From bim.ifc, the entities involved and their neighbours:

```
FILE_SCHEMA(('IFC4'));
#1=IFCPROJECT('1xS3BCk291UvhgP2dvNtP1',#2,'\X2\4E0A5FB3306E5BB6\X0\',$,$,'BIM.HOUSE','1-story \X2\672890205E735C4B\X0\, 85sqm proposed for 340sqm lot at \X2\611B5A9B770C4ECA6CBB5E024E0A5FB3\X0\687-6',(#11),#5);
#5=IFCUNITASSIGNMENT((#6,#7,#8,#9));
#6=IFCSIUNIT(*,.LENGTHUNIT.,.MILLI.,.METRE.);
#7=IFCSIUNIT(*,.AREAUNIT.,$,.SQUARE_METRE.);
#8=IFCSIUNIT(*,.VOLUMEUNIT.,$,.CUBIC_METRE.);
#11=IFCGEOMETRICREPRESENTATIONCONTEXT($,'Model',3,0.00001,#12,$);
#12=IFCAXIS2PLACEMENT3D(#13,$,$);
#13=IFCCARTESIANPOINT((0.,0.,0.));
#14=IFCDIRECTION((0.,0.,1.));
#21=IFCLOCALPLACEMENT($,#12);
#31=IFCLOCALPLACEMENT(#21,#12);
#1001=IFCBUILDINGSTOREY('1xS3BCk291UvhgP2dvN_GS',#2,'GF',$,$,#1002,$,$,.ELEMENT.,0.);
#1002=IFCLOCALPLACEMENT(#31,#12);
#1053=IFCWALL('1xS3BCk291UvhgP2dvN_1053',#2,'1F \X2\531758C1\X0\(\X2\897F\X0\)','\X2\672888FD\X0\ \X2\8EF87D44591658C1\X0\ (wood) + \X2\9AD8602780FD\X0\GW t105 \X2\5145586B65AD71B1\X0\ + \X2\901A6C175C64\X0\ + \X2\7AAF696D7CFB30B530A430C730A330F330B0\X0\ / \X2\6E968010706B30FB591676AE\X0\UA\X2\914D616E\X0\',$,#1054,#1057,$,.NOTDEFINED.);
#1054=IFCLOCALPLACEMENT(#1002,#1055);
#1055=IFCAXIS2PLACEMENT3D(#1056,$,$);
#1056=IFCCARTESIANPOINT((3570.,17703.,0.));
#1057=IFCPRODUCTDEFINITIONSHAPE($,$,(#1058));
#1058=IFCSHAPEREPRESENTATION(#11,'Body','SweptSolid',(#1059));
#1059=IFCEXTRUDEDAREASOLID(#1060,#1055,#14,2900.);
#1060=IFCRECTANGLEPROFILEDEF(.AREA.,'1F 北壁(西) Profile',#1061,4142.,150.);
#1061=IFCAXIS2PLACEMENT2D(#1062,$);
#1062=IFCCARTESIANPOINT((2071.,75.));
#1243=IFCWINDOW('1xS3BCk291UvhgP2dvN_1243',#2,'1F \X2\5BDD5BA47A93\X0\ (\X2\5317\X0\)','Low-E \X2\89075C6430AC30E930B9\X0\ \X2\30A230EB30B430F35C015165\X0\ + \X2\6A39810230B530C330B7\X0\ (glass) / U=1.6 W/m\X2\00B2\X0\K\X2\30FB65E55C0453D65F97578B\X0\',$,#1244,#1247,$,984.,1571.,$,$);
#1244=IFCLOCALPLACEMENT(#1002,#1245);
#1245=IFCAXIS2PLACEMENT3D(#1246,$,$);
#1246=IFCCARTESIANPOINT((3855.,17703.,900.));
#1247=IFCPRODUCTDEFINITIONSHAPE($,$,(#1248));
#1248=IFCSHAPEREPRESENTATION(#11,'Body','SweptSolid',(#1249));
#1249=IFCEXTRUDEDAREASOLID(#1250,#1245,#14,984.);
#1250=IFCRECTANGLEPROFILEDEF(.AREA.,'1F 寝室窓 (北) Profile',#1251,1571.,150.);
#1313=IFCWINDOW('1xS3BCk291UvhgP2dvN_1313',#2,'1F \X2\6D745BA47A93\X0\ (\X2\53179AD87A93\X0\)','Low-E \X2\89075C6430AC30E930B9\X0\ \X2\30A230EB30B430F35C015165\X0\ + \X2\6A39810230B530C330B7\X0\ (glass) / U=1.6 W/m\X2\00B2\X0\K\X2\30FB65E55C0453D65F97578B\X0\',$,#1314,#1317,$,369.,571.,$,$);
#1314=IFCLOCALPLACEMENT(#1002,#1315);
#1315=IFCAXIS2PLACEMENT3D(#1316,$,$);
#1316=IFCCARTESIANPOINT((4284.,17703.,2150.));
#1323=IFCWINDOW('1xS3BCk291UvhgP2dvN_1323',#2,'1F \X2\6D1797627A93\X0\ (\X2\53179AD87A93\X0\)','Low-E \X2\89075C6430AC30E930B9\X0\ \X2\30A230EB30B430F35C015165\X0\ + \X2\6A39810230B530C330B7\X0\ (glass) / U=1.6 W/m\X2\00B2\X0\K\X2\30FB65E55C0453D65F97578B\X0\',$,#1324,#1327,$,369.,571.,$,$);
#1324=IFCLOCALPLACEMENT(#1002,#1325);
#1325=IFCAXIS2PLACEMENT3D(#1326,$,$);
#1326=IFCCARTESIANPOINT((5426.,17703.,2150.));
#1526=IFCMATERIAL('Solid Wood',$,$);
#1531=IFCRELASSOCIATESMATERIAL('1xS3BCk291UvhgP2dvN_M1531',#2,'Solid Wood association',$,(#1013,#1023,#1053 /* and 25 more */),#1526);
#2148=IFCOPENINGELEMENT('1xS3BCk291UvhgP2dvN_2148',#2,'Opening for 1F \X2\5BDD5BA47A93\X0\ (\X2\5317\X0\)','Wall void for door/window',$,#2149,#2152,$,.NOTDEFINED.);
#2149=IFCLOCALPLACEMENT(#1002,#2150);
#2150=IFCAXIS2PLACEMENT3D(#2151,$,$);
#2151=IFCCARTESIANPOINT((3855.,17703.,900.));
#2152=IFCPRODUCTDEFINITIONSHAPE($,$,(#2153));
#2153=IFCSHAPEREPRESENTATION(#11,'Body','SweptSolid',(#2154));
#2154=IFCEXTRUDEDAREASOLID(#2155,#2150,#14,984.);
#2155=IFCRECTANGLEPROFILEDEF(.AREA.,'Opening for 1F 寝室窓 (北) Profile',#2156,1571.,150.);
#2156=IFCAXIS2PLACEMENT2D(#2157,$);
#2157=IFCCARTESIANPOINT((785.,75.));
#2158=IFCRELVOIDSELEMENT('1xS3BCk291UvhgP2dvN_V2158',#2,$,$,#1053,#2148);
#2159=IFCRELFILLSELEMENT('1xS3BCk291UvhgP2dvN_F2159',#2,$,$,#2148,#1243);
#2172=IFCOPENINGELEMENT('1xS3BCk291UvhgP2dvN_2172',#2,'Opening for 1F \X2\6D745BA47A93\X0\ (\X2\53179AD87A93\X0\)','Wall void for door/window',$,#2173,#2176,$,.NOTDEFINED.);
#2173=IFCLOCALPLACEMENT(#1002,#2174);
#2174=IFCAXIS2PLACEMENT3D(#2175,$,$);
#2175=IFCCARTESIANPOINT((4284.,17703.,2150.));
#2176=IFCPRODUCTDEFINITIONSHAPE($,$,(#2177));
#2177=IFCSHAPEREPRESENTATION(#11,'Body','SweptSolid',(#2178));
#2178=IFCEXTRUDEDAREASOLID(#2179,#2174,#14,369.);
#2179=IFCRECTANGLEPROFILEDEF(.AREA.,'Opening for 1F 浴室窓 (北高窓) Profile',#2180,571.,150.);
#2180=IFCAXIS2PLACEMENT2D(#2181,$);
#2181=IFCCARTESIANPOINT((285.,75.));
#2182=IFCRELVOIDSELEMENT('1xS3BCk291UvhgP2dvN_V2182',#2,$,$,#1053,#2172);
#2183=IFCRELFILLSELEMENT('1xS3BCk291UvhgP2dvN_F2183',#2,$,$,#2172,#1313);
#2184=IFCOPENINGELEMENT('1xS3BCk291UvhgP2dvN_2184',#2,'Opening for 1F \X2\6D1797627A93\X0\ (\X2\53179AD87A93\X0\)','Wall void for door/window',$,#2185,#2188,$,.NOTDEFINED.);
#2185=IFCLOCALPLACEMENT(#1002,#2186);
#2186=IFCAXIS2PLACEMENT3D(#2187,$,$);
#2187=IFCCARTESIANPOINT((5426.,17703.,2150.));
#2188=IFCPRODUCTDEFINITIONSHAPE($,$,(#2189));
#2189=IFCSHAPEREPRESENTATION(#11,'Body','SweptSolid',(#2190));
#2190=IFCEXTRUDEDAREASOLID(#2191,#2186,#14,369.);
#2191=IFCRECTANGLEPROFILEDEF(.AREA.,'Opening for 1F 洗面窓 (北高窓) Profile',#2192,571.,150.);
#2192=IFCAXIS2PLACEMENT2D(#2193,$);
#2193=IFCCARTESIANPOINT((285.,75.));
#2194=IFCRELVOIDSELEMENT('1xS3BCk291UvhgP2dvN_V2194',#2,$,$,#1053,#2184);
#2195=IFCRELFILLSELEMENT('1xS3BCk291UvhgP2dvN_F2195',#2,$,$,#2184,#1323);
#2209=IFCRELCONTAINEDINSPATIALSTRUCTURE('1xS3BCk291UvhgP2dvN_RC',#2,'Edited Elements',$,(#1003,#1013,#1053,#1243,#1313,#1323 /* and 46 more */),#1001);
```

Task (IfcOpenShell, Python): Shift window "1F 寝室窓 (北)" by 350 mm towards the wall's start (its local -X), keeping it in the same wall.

```python
import ifcopenshell
import ifcopenshell.api.geometry
import ifcopenshell.util.placement
import ifcopenshell.util.unit

model = ifcopenshell.open("bim.ifc")
unit_scale = ifcopenshell.util.unit.calculate_unit_scale(model)

window = model.by_guid("1xS3BCk291UvhgP2dvN_1243")
opening = window.FillsVoids[0].RelatingOpeningElement
wall = opening.VoidsElements[0].RelatingBuildingElement

wall_matrix = ifcopenshell.util.placement.get_local_placement(wall.ObjectPlacement)
shift = wall_matrix[:3, 0] * -0.35 / unit_scale
before = ifcopenshell.util.placement.get_local_placement(window.ObjectPlacement)[:3, 3].copy()

# The window is not placed relative to its opening, so move both.
for product in (opening, window):
    matrix = ifcopenshell.util.placement.get_local_placement(product.ObjectPlacement)
    matrix[:3, 3] += shift
    ifcopenshell.api.geometry.edit_object_placement(model, product=product, matrix=matrix, is_si=False)

after = ifcopenshell.util.placement.get_local_placement(window.ObjectPlacement)[:3, 3]
print("window moved by", (after - before).round(3) + 0.0)

model.write("bim_edited.ifc")
```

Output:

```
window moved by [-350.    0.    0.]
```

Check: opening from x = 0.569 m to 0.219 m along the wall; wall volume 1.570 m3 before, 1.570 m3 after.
